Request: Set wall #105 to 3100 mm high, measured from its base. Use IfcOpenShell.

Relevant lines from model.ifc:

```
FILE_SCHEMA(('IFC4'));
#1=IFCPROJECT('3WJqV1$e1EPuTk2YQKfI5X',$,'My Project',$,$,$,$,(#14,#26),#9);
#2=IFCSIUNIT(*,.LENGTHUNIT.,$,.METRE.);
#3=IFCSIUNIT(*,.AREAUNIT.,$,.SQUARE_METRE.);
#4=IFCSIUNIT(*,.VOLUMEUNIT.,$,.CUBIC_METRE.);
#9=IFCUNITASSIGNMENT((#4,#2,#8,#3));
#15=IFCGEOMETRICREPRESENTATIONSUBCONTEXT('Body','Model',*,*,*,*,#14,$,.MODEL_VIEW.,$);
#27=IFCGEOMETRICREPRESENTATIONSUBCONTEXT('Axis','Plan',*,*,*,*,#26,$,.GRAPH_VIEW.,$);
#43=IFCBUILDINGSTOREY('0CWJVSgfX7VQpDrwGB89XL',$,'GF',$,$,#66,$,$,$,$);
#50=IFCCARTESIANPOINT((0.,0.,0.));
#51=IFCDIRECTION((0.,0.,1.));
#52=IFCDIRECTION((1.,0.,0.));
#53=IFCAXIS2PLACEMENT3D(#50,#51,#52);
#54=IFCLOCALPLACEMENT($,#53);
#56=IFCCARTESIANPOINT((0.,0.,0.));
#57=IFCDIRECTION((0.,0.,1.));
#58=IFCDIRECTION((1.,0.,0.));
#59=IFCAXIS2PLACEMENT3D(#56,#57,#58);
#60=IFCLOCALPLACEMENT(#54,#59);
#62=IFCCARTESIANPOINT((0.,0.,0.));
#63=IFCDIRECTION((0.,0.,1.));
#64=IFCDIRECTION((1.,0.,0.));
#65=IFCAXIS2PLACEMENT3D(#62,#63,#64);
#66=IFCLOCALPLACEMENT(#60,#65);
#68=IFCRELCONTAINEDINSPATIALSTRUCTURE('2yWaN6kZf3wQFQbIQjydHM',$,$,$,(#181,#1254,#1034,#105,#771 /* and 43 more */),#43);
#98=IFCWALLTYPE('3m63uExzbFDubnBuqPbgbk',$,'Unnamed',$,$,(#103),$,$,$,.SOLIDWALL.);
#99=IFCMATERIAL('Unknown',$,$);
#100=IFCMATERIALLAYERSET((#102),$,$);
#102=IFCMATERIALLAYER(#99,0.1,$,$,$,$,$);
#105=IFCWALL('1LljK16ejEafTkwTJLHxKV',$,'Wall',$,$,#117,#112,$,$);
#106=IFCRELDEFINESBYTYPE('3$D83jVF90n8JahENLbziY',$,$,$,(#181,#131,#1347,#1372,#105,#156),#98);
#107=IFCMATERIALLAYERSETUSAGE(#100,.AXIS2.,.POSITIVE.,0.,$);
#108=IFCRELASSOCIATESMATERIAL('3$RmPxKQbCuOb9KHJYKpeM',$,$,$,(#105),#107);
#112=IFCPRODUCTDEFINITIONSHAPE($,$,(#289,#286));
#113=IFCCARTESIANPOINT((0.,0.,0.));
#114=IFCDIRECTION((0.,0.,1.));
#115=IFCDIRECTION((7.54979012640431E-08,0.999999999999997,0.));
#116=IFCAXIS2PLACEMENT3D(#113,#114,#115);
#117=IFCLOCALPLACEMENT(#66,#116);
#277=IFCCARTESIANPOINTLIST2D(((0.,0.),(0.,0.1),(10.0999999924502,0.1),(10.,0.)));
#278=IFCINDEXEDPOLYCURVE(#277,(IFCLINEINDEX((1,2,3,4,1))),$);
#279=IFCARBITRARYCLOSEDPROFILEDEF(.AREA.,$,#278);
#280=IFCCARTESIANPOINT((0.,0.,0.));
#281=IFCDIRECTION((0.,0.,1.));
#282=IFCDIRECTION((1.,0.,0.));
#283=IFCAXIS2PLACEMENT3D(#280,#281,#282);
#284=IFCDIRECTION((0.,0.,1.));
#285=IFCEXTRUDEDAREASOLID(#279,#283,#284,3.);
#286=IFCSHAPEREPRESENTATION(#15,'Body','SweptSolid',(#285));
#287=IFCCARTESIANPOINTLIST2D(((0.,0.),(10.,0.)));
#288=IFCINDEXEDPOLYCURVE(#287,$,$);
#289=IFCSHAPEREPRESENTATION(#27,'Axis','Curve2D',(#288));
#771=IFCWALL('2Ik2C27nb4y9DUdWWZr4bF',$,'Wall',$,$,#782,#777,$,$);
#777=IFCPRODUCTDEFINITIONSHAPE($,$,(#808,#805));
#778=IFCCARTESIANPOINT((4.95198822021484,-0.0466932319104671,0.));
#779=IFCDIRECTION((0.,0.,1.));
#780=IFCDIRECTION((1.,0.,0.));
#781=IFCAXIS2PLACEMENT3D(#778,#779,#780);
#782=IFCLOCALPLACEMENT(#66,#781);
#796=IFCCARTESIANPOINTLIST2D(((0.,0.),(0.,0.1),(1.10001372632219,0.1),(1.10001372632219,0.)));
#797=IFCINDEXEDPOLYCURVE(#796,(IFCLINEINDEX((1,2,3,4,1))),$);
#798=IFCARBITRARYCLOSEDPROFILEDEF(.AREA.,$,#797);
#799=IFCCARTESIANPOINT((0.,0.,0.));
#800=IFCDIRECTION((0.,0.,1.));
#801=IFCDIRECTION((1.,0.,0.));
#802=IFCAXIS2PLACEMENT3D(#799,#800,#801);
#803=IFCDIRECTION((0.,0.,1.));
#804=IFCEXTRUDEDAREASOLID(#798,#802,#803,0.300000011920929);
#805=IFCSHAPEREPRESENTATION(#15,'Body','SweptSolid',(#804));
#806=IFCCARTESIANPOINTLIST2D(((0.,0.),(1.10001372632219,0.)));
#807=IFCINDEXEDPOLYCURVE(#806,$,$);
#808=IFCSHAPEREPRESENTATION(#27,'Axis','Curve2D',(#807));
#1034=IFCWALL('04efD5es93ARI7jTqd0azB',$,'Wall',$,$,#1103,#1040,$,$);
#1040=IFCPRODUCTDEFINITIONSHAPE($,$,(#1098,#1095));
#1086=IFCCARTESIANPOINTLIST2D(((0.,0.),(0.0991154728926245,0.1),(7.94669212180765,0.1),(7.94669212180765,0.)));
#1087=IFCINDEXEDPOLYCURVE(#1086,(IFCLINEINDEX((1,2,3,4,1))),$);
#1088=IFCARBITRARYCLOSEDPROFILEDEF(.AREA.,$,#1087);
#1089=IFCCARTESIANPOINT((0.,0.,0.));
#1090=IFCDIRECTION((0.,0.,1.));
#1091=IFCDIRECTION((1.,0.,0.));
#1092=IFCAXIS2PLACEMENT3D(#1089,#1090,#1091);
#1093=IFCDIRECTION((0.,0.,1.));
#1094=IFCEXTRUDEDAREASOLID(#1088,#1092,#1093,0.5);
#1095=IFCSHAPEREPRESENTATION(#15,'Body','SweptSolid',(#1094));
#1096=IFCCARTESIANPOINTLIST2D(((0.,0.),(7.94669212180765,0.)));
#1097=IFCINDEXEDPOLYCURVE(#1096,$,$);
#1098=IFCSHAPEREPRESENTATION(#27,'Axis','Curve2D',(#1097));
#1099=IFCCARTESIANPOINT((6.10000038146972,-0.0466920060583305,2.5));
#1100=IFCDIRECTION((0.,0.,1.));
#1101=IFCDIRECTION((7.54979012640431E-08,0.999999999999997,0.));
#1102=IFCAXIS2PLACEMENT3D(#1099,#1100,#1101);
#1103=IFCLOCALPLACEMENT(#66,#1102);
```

```python
import ifcopenshell
import ifcopenshell.geom
import ifcopenshell.util.representation
import ifcopenshell.util.shape

model = ifcopenshell.open("model.ifc")
settings = ifcopenshell.geom.settings()


def volume(element):
    """Net volume in cubic metres, openings subtracted."""
    shape = ifcopenshell.geom.create_shape(settings, element)
    return ifcopenshell.util.shape.get_volume(shape.geometry)


wall = model.by_guid("1LljK16ejEafTkwTJLHxKV")
before = volume(wall)

body = ifcopenshell.util.representation.get_representation(wall, "Model", "Body")
solid = body.Items[0]
old_height = solid.Depth
solid.Depth = 3.1
after = volume(wall)

print(f"height {old_height:g} -> {solid.Depth:g}, volume {before:.3f} -> {after:.3f} m3")

model.write("model_edited.ifc")
```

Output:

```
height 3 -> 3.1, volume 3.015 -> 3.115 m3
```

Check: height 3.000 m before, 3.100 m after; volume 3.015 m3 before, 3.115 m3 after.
